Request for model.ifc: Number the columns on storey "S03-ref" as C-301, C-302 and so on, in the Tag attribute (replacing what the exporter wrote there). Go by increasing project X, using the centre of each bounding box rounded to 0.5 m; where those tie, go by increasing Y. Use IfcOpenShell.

First a look at what the model holds.

```python
import ifcopenshell
import ifcopenshell.util.element
import ifcopenshell.util.placement

model = ifcopenshell.open("model.ifc")
print(model.schema)
storey = next(s for s in model.by_type("IfcBuildingStorey") if s.Name == "S03-ref")
columns = [e for e in ifcopenshell.util.element.get_decomposition(storey) if e.is_a("IfcColumn")]
for e in sorted(columns, key=lambda e: e.id()):
    origin = ifcopenshell.util.placement.get_local_placement(e.ObjectPlacement)[:3, 3]
    print(e.id(), e.Tag, e.Name, origin.round(2) + 0.0, sep=" | ")
```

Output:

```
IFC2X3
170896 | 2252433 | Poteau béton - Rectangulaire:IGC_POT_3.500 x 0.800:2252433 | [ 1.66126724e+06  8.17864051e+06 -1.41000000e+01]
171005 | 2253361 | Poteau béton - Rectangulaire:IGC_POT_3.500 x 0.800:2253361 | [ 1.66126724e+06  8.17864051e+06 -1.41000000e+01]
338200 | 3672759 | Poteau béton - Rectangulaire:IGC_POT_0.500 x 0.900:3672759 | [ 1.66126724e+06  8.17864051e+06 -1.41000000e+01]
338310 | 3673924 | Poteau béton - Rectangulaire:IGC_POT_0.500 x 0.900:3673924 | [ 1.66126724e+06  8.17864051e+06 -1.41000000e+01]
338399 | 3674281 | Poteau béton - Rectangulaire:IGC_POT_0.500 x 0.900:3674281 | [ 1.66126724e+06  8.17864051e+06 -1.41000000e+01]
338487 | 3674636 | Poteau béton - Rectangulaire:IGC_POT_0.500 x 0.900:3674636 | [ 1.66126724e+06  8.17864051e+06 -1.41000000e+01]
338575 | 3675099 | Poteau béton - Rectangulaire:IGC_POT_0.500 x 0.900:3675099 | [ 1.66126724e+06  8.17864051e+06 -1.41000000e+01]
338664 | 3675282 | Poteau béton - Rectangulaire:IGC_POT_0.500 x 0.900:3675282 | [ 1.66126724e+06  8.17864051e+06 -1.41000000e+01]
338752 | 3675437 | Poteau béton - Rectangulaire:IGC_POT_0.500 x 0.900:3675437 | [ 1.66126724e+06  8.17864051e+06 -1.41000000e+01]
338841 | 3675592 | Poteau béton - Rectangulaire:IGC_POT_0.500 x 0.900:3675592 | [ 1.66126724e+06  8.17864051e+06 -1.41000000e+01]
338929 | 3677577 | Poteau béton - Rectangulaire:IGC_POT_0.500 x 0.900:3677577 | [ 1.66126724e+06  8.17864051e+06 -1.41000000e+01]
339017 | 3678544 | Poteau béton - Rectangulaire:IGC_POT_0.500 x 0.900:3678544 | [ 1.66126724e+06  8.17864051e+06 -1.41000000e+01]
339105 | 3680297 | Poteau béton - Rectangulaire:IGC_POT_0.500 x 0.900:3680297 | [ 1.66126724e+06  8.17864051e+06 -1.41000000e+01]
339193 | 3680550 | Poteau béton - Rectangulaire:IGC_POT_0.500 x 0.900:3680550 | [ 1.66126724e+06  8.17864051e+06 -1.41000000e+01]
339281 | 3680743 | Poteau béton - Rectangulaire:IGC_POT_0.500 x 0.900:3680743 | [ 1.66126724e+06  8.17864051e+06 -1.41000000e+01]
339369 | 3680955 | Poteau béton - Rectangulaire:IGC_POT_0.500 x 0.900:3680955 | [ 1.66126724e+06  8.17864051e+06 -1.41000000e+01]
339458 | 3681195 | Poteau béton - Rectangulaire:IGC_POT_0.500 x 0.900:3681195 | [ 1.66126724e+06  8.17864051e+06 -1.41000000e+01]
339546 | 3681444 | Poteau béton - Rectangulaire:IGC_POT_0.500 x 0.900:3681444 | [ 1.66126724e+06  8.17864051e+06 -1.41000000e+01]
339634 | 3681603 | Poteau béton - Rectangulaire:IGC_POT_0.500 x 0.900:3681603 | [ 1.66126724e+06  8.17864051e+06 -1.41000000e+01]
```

```python
import ifcopenshell
import ifcopenshell.geom
import ifcopenshell.util.element
import ifcopenshell.util.shape

model = ifcopenshell.open("model.ifc")
settings = ifcopenshell.geom.settings()
settings.set("use-world-coords", True)


def centre(element):
    shape = ifcopenshell.geom.create_shape(settings, element)
    return ifcopenshell.util.shape.get_bbox_centroid(shape.geometry)


storey = next(s for s in model.by_type("IfcBuildingStorey") if s.Name == "S03-ref")
columns = [e for e in ifcopenshell.util.element.get_decomposition(storey) if e.is_a("IfcColumn")]

# Insertion points can sit at a corner or the storey origin, so sort by the geometry (in metres).
centres = {e: centre(e) for e in columns}
columns.sort(key=lambda e: (round(centres[e][0] / 0.5), centres[e][1]))

for i, e in enumerate(columns, start=1):
    number = f"C-3{i:02d}"
    e.Tag = number
    print(e.id(), number)

model.write("model_updated.ifc")
```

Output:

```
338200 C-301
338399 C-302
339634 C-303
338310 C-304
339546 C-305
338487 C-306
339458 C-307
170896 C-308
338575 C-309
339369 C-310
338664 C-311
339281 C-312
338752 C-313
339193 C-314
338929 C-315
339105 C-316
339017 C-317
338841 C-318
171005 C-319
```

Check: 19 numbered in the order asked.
